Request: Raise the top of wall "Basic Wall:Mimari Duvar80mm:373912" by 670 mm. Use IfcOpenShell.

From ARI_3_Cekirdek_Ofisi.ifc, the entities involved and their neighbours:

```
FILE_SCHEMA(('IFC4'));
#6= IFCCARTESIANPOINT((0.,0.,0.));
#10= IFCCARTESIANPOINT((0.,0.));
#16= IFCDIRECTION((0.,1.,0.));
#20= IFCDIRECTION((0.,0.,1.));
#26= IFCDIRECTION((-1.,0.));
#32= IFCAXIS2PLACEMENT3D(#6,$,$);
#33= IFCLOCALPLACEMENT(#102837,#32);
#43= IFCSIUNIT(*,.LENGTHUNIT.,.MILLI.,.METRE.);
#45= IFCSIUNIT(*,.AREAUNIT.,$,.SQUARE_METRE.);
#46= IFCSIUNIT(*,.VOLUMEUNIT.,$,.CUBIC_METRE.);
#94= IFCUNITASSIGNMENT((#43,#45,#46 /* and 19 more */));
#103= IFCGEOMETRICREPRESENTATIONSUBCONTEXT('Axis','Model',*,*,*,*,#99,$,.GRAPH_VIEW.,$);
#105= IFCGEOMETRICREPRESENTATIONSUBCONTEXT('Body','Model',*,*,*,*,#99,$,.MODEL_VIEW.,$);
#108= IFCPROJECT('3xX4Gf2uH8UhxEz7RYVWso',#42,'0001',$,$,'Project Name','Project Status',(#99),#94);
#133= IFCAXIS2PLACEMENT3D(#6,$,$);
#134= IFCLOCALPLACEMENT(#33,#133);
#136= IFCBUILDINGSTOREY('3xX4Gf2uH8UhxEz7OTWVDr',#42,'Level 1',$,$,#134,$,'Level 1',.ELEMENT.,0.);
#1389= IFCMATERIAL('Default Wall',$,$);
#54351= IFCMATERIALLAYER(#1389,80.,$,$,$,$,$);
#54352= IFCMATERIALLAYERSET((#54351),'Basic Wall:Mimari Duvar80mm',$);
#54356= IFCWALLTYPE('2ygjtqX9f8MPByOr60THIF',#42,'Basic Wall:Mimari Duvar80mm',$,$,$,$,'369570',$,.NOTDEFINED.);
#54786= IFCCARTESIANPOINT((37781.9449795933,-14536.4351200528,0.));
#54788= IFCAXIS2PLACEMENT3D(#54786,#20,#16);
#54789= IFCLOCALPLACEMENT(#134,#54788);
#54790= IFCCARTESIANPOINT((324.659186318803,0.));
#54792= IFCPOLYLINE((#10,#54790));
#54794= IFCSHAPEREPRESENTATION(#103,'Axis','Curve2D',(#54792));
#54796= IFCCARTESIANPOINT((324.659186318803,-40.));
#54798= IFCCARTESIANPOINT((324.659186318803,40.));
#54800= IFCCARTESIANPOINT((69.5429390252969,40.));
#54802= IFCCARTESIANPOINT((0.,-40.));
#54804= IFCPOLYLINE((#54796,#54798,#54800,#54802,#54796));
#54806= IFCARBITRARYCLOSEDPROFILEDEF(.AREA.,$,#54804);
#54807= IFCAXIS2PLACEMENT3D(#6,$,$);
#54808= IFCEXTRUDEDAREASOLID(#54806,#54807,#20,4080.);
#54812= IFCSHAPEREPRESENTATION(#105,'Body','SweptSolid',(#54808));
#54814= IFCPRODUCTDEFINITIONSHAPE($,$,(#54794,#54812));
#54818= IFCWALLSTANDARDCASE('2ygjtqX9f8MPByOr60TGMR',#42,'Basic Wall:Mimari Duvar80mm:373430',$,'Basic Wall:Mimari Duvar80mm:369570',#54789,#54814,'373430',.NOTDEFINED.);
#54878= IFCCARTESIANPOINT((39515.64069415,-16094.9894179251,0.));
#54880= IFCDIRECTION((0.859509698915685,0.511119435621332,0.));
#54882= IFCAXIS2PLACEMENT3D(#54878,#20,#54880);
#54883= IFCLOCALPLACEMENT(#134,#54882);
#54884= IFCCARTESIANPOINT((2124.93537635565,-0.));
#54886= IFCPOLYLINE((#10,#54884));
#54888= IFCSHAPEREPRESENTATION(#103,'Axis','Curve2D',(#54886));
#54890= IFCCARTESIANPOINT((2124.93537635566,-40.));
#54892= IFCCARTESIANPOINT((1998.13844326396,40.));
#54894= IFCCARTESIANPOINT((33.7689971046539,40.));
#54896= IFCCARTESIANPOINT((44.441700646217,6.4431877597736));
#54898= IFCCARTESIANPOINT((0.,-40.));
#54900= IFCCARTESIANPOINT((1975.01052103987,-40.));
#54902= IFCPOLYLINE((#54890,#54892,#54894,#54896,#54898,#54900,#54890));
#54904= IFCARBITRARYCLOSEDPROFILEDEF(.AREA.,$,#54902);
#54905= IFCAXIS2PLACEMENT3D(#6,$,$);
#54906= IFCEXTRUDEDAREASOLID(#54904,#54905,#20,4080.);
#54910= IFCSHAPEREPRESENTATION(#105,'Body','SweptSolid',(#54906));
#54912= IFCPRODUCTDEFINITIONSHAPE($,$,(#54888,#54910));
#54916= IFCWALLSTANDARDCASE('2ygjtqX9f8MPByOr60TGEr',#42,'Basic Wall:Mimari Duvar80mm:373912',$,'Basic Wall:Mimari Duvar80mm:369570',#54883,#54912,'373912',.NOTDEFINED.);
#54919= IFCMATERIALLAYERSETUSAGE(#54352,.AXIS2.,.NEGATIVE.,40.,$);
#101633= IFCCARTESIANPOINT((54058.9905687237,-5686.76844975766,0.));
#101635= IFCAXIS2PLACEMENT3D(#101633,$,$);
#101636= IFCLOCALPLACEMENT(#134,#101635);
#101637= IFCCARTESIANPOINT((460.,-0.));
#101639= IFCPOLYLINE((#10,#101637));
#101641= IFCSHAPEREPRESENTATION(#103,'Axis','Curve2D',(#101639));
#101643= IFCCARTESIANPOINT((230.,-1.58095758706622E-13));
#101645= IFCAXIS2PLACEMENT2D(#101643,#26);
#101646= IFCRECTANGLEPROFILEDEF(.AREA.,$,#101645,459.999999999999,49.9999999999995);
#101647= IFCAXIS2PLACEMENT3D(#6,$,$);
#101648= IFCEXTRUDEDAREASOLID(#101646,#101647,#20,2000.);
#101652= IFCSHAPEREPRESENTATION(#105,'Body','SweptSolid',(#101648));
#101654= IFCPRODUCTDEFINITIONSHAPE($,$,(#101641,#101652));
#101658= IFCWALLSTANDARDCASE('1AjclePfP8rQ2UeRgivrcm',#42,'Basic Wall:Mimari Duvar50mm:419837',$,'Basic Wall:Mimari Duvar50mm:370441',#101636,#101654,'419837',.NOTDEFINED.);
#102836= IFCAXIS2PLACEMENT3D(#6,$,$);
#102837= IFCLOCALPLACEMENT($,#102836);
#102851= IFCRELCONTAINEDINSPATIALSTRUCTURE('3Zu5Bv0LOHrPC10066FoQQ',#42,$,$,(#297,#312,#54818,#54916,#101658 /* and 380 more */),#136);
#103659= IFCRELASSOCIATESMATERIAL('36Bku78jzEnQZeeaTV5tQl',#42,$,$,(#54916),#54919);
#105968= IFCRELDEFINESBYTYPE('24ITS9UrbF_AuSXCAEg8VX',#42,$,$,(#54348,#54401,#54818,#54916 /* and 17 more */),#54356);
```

```python
import ifcopenshell
import ifcopenshell.geom
import ifcopenshell.util.representation
import ifcopenshell.util.shape
import ifcopenshell.util.unit

model = ifcopenshell.open("ARI_3_Cekirdek_Ofisi.ifc")
unit_scale = ifcopenshell.util.unit.calculate_unit_scale(model)
settings = ifcopenshell.geom.settings()


def volume(element):
    """Net volume in cubic metres, openings subtracted."""
    shape = ifcopenshell.geom.create_shape(settings, element)
    return ifcopenshell.util.shape.get_volume(shape.geometry)


wall = model.by_guid("2ygjtqX9f8MPByOr60TGEr")
before = volume(wall)

body = ifcopenshell.util.representation.get_representation(wall, "Model", "Body")
solid = body.Items[0]
old_height = solid.Depth
solid.Depth += 0.67 / unit_scale
after = volume(wall)

print(f"height {old_height:g} -> {solid.Depth:g}, volume {before:.3f} -> {after:.3f} m3")

model.write("ARI_3_Cekirdek_Ofisi_v2.ifc")
```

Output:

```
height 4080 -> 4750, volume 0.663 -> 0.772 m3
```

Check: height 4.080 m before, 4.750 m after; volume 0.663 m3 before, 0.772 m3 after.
